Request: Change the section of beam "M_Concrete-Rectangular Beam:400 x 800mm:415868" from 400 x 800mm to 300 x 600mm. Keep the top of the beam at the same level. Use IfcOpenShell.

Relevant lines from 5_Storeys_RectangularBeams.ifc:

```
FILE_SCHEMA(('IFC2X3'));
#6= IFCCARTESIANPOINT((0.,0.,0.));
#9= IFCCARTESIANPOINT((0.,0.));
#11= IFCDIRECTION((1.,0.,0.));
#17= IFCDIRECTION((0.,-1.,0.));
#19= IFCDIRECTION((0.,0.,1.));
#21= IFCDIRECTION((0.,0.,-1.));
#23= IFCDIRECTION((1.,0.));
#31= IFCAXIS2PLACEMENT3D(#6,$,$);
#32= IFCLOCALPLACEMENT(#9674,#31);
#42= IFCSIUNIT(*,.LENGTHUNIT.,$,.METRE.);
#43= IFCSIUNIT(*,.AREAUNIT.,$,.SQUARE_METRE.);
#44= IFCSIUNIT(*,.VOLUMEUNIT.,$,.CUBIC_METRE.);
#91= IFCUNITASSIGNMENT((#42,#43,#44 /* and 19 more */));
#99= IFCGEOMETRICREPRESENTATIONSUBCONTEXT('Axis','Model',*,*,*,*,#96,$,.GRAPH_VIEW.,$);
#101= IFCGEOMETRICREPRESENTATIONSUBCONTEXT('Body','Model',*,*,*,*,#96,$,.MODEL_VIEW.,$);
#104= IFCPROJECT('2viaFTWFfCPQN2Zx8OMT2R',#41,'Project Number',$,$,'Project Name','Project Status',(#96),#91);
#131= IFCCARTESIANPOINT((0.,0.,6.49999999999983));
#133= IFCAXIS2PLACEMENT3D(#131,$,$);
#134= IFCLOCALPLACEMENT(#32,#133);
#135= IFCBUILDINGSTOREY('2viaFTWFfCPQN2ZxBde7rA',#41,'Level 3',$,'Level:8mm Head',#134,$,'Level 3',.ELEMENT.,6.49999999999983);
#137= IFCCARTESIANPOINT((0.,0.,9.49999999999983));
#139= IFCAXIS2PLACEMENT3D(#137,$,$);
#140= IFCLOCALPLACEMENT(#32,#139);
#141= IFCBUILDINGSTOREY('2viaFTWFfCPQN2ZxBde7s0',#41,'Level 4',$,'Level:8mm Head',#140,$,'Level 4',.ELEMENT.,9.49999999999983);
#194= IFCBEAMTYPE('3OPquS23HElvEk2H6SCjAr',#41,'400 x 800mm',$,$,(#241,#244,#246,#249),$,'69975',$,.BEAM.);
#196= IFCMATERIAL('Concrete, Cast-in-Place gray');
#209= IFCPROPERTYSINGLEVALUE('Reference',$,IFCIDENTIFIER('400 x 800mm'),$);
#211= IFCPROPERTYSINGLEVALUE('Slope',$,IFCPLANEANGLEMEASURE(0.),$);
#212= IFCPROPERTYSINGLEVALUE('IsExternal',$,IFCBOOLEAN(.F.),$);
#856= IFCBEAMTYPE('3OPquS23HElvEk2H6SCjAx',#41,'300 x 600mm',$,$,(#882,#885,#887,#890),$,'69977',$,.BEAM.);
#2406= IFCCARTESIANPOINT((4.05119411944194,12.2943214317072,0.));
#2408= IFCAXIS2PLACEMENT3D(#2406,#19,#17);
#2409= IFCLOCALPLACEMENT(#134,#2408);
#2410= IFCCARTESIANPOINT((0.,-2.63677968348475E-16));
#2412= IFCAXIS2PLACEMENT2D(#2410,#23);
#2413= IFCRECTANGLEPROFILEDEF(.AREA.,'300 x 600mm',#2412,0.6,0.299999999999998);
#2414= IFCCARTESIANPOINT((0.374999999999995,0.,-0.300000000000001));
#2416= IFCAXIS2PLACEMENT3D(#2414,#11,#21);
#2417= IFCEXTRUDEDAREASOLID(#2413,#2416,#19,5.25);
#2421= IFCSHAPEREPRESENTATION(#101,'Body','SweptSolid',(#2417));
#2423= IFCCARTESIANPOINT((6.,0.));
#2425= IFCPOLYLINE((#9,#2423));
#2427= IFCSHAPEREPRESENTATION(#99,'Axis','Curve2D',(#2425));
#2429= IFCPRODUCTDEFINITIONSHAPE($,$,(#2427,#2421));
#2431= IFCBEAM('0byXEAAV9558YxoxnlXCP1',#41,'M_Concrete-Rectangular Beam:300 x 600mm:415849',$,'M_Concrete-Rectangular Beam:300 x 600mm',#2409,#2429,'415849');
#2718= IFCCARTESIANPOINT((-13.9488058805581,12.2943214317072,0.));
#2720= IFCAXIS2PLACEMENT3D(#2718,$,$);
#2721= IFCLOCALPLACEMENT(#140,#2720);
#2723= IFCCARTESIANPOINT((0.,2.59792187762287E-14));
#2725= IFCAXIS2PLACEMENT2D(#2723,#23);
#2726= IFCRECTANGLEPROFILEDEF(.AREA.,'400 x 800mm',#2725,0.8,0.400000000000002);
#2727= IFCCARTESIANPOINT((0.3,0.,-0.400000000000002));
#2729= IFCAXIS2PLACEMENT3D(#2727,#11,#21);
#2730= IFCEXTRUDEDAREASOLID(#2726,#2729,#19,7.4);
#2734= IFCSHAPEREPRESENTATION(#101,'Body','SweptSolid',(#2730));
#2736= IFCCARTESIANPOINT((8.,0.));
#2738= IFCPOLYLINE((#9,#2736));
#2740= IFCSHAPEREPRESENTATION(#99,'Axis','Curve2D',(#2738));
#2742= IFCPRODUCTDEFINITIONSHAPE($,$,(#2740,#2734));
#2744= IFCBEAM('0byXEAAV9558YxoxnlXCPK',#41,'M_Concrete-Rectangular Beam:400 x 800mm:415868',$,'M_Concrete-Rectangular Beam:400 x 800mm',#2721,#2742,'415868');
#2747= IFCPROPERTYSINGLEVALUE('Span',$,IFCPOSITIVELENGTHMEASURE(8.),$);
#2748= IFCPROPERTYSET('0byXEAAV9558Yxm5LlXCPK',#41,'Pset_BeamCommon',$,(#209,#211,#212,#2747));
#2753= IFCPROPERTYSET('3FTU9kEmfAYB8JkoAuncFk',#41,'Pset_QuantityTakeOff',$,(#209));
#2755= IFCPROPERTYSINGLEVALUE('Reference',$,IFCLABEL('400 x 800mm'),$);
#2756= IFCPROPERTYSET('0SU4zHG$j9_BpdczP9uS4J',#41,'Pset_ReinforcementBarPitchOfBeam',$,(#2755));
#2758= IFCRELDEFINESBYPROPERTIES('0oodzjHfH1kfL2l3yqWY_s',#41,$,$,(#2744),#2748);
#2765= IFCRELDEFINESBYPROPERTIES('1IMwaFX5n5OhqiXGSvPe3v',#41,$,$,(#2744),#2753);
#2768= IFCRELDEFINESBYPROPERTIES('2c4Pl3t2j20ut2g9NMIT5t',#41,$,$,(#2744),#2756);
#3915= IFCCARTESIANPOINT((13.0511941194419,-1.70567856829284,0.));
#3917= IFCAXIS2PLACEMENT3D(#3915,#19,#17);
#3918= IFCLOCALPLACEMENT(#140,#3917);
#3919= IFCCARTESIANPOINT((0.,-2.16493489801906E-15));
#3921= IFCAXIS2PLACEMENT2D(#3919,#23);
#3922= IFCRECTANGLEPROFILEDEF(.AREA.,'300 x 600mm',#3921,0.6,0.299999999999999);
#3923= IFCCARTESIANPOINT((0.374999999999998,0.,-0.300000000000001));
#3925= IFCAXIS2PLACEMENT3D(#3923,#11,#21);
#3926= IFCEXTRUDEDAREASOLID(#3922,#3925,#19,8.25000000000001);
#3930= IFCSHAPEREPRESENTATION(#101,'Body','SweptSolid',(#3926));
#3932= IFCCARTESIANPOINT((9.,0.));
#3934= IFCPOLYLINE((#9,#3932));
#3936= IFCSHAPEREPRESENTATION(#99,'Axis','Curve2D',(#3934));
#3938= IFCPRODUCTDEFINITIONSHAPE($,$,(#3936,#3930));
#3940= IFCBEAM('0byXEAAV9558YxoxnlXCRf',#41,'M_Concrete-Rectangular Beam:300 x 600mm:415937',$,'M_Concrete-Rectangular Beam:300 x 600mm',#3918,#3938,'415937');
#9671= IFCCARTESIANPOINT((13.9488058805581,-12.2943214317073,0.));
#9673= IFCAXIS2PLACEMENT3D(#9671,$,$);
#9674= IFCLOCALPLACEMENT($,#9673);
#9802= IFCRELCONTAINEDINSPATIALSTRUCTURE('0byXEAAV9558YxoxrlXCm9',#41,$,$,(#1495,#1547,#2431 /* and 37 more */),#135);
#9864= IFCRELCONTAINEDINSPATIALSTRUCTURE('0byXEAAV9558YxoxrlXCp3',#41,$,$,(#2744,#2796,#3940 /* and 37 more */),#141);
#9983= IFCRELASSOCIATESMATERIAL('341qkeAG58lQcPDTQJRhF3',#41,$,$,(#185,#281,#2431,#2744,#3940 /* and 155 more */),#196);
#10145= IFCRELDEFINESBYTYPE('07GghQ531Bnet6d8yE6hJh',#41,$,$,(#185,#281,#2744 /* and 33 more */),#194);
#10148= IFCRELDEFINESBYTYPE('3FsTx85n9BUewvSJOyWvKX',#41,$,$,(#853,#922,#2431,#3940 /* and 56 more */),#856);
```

```python
import ifcopenshell
import ifcopenshell.api.pset
import ifcopenshell.api.type
import ifcopenshell.util.element
import ifcopenshell.util.representation

model = ifcopenshell.open("5_Storeys_RectangularBeams.ifc")

member = model.by_guid("0byXEAAV9558YxoxnlXCPK")
source = next(p for p in model.by_type("IfcRectangleProfileDef") if p.ProfileName == "300 x 600mm")

body = ifcopenshell.util.representation.get_representation(member, "Model", "Body")
solid = body.Items[0]
old_profile = solid.SweptArea

# Copy the section's sizes but keep this member's own profile position.
profile = ifcopenshell.util.element.copy(model, source)
# Profiles are centred, so shift by half the change in depth to hold the top.
shift = (old_profile.XDim - profile.XDim) / 2
x, y = old_profile.Position.Location.Coordinates
up = (-1.0, 0.0)  # upwards, in the solid's own plane
location = model.createIfcCartesianPoint((x + up[0] * shift, y + up[1] * shift))
profile.Position = model.createIfcAxis2Placement2D(location, old_profile.Position.RefDirection)
solid.SweptArea = profile
if not model.get_total_inverses(old_profile):
    ifcopenshell.util.element.remove_deep2(model, old_profile)

new_type = model.by_guid("3OPquS23HElvEk2H6SCjAx")
ifcopenshell.api.type.assign_type(
    model, related_objects=[member], relating_type=new_type, should_map_representations=False
)
member.Name = member.Name.replace("400 x 800mm", "300 x 600mm")
member.ObjectType = "M_Concrete-Rectangular Beam:300 x 600mm"
pset = model.by_id(ifcopenshell.util.element.get_pset(member, "Pset_BeamCommon", should_inherit=False)["id"])
ifcopenshell.api.pset.edit_pset(model, pset=pset, properties={"Reference": "300 x 600mm"})
pset = model.by_id(ifcopenshell.util.element.get_pset(member, "Pset_QuantityTakeOff", should_inherit=False)["id"])
ifcopenshell.api.pset.edit_pset(model, pset=pset, properties={"Reference": "300 x 600mm"})
pset = model.by_id(ifcopenshell.util.element.get_pset(member, "Pset_ReinforcementBarPitchOfBeam", should_inherit=False)["id"])
ifcopenshell.api.pset.edit_pset(model, pset=pset, properties={"Reference": "300 x 600mm"})

print(solid.SweptArea)

model.write("5_Storeys_RectangularBeams-out.ifc")
```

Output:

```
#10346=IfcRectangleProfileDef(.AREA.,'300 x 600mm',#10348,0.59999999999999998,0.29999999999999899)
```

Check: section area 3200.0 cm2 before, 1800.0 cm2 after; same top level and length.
